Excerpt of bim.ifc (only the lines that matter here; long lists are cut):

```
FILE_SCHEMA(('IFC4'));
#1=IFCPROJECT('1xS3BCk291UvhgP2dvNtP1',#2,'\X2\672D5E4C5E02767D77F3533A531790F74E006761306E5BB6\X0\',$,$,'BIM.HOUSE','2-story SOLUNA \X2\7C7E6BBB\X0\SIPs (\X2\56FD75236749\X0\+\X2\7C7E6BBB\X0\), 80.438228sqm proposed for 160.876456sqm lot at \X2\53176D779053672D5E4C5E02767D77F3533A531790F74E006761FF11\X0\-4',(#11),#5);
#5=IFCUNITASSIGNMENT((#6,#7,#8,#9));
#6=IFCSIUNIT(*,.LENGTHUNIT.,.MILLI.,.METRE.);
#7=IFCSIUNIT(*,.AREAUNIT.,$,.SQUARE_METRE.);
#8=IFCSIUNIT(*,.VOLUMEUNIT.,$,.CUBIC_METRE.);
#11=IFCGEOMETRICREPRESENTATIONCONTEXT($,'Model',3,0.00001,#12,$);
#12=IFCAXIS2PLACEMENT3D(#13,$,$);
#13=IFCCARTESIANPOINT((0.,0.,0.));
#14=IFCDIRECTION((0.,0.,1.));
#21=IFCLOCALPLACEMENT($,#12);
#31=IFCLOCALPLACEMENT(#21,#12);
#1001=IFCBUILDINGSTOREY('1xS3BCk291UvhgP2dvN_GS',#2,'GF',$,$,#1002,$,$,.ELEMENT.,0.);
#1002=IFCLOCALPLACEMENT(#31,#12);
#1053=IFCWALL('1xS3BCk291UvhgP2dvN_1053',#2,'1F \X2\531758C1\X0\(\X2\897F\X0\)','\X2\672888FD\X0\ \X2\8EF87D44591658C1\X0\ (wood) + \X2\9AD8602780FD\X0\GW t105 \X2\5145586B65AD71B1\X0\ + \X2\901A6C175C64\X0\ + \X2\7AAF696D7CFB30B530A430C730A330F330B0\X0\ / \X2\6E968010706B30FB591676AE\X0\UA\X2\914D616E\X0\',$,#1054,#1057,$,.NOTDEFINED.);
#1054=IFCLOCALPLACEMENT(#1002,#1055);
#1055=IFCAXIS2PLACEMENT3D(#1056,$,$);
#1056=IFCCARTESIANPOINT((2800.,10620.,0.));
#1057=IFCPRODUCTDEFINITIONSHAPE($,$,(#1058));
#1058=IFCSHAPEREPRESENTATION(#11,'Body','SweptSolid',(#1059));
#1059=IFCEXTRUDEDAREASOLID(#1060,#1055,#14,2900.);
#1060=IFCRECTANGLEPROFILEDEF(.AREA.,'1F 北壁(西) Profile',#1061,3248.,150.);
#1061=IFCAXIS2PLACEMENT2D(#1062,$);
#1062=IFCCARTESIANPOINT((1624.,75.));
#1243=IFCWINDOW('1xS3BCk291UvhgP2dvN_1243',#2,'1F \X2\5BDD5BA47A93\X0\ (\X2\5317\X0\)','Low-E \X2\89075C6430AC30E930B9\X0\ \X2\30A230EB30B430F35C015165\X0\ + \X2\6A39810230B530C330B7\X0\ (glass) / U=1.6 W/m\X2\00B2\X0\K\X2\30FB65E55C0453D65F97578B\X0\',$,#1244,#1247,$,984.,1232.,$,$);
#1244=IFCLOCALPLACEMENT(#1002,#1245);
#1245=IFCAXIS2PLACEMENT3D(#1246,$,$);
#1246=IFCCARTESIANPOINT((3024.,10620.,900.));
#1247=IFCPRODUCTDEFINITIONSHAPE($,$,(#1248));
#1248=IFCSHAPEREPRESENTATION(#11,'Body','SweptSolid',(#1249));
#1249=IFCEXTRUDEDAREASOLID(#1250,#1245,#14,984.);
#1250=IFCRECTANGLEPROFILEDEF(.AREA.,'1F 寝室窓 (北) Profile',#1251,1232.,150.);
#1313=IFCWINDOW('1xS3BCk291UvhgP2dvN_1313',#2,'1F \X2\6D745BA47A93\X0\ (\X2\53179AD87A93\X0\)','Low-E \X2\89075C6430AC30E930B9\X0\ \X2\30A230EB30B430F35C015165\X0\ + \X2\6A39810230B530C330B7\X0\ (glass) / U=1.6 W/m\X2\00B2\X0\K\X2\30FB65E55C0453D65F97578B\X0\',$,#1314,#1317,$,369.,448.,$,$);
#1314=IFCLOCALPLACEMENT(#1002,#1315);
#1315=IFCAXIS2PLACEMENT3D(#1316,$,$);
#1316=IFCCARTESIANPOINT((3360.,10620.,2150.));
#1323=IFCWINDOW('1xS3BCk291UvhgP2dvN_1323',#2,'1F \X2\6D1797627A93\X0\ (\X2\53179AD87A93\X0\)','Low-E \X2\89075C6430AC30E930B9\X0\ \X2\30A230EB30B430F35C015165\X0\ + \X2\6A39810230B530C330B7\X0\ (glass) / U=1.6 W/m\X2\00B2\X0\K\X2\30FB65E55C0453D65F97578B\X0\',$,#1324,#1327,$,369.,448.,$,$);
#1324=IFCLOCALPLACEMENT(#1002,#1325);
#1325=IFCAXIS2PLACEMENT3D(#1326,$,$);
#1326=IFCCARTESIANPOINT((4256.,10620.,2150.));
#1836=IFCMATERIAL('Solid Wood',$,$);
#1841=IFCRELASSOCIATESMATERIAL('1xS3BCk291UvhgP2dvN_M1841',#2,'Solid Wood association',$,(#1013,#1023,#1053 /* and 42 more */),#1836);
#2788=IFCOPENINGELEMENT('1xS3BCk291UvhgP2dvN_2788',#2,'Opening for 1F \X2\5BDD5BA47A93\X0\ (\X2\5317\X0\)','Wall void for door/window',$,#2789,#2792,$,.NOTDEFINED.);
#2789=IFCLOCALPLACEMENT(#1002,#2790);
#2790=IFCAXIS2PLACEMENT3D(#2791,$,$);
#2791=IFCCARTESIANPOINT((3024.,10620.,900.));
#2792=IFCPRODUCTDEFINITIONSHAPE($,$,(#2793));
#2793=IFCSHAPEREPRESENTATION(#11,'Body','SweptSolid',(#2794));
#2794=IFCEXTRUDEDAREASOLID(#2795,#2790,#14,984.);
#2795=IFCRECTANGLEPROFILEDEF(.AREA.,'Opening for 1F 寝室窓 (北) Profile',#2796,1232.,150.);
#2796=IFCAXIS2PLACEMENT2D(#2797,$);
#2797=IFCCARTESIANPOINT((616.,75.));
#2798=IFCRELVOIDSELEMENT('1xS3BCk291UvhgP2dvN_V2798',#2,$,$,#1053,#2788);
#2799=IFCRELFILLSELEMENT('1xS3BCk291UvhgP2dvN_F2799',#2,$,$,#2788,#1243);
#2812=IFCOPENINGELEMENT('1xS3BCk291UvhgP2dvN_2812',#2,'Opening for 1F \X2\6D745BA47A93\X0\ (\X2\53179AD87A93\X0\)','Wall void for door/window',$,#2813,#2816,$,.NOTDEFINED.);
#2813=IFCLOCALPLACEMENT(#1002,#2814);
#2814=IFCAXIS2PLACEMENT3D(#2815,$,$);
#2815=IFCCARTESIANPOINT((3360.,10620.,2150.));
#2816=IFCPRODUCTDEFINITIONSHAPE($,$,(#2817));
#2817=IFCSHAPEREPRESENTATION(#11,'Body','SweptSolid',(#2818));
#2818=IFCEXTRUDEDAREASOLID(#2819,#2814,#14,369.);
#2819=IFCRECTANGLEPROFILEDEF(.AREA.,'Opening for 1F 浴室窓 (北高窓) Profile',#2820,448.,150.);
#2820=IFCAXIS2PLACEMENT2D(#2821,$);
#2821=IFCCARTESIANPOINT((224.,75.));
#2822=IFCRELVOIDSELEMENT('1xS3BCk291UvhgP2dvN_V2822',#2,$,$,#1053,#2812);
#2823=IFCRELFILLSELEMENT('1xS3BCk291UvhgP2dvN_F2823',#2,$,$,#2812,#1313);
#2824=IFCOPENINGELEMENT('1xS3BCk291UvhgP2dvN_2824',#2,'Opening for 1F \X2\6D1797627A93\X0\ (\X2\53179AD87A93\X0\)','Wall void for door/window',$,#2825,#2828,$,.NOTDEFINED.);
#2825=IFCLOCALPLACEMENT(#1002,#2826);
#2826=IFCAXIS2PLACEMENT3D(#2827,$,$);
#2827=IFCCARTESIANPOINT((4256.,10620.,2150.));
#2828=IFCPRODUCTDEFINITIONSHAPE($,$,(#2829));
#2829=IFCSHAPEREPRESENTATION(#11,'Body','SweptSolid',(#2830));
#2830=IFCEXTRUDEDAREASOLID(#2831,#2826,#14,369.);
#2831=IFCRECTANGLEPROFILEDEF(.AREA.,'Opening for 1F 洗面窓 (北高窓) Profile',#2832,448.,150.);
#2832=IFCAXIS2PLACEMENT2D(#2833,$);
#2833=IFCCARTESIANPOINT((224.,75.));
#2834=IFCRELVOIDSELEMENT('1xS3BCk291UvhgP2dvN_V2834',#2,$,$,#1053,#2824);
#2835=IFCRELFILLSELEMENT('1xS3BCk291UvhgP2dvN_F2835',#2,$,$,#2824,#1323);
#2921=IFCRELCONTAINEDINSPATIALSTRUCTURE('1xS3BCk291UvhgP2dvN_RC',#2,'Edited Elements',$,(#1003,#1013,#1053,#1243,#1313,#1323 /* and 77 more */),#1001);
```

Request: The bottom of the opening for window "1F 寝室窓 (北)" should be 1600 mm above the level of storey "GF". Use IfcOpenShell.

```python
import numpy as np
import ifcopenshell
import ifcopenshell.api.geometry
import ifcopenshell.geom
import ifcopenshell.util.element
import ifcopenshell.util.placement
import ifcopenshell.util.shape
import ifcopenshell.util.unit

model = ifcopenshell.open("bim.ifc")
unit_scale = ifcopenshell.util.unit.calculate_unit_scale(model)

window = model.by_id(1243)
opening = window.FillsVoids[0].RelatingOpeningElement
storey = ifcopenshell.util.element.get_container(window, ifc_class="IfcBuildingStorey")
level = ifcopenshell.util.placement.get_local_placement(storey.ObjectPlacement)[2, 3]

# The opening's origin need not be at the sill, so measure its lowest point.
shape = ifcopenshell.geom.create_shape(ifcopenshell.geom.settings(), opening)
bottom = ifcopenshell.util.shape.get_shape_bottom_elevation(shape, shape.geometry) / unit_scale
dz = level + 1.6 / unit_scale - bottom

shift = np.array([0.0, 0.0, dz])
# The window is not placed relative to its opening, so move both.
for product in (opening, window):
    matrix = ifcopenshell.util.placement.get_local_placement(product.ObjectPlacement)
    matrix[:3, 3] += shift
    ifcopenshell.api.geometry.edit_object_placement(model, product=product, matrix=matrix, is_si=False)

print(f"moved by {dz * unit_scale:+.3f} m")

model.write("bim_updated.ifc")
```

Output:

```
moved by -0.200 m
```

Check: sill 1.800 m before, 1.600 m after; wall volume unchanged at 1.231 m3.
